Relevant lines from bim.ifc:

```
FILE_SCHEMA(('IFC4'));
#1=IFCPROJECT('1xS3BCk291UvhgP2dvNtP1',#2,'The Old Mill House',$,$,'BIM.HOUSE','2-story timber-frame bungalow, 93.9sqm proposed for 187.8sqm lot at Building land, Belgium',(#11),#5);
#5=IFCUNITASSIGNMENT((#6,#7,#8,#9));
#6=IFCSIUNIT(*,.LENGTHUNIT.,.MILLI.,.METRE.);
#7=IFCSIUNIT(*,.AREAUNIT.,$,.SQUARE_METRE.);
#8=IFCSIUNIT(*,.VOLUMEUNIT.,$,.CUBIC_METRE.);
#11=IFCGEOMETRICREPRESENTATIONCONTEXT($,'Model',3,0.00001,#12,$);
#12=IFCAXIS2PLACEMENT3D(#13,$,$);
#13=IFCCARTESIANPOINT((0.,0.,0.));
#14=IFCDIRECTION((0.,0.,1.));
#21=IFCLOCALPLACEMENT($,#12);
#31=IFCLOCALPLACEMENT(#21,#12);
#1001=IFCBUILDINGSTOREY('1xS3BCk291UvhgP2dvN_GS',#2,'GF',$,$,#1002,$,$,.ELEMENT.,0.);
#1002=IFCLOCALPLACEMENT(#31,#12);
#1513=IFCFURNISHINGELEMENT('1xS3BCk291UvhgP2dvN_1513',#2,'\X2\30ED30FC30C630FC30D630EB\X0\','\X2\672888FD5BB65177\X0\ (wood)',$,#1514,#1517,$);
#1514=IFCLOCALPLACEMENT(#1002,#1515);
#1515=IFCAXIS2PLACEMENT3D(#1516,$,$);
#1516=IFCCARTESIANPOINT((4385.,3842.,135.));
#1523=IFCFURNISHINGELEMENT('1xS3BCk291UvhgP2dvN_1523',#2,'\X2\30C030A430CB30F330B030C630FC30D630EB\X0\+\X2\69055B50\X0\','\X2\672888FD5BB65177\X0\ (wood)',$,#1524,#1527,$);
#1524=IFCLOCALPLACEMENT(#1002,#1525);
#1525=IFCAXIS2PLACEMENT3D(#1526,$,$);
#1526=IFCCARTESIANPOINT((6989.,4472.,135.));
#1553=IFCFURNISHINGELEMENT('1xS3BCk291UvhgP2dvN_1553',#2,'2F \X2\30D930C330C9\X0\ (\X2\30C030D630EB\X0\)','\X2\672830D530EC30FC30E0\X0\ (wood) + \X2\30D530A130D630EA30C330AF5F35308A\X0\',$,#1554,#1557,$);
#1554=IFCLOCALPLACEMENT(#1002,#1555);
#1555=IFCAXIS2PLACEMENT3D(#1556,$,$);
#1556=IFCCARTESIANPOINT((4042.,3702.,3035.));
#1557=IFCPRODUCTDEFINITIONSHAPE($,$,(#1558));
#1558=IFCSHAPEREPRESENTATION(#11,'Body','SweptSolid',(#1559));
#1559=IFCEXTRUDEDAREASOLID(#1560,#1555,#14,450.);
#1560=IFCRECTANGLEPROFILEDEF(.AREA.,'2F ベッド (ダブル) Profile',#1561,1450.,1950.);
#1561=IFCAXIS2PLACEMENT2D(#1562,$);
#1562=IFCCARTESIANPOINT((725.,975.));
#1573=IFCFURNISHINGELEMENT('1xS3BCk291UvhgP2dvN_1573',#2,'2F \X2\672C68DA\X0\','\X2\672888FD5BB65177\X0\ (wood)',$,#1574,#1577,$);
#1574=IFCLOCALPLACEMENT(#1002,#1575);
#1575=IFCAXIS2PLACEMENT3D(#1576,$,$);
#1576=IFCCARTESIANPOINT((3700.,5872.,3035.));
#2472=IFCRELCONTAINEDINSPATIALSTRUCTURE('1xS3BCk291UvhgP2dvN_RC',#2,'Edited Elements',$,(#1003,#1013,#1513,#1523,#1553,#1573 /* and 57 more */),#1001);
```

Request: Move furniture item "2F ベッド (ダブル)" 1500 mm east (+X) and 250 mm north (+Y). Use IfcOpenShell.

```python
import ifcopenshell
import ifcopenshell.api.geometry
import ifcopenshell.util.placement
import ifcopenshell.util.unit

model = ifcopenshell.open("bim.ifc")
unit_scale = ifcopenshell.util.unit.calculate_unit_scale(model)

item = model.by_guid("1xS3BCk291UvhgP2dvN_1553")
matrix = ifcopenshell.util.placement.get_local_placement(item.ObjectPlacement)
matrix[0, 3] += 1.5 / unit_scale
matrix[1, 3] += 0.25 / unit_scale
ifcopenshell.api.geometry.edit_object_placement(model, product=item, matrix=matrix, is_si=False)

print(ifcopenshell.util.placement.get_local_placement(item.ObjectPlacement).round(3) + 0.0)

model.write("bim_v2.ifc")
```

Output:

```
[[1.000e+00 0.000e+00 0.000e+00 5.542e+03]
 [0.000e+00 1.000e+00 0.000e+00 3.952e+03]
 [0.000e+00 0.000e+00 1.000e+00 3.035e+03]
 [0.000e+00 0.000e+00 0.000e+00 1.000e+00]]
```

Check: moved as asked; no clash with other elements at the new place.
